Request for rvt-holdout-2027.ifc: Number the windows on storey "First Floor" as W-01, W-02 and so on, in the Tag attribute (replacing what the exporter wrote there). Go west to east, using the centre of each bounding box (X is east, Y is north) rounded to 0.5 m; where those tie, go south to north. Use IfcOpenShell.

First a look at what the model holds.

```python
import ifcopenshell
import ifcopenshell.util.element
import ifcopenshell.util.placement

model = ifcopenshell.open("rvt-holdout-2027.ifc")
print(model.schema)
storey = next(s for s in model.by_type("IfcBuildingStorey") if s.Name == "First Floor")
windows = [e for e in ifcopenshell.util.element.get_decomposition(storey) if e.is_a("IfcWindow")]
for e in sorted(windows, key=lambda e: e.id()):
    origin = ifcopenshell.util.placement.get_local_placement(e.ObjectPlacement)[:3, 3]
    print(e.id(), e.Tag, e.Name, origin.round(2) + 0.0, sep=" | ")
```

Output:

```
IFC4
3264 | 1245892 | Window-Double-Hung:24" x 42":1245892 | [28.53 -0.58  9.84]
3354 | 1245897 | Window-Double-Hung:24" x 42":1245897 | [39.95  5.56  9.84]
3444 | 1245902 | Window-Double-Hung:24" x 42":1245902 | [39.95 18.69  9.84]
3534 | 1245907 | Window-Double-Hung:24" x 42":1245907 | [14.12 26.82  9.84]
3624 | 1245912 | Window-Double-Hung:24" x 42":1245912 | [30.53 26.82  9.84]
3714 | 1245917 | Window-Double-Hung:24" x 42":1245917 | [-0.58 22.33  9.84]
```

```python
import ifcopenshell
import ifcopenshell.geom
import ifcopenshell.util.element
import ifcopenshell.util.shape

model = ifcopenshell.open("rvt-holdout-2027.ifc")
settings = ifcopenshell.geom.settings()
settings.set("use-world-coords", True)


def centre(element):
    shape = ifcopenshell.geom.create_shape(settings, element)
    return ifcopenshell.util.shape.get_bbox_centroid(shape.geometry)


storey = next(s for s in model.by_type("IfcBuildingStorey") if s.Name == "First Floor")
windows = [e for e in ifcopenshell.util.element.get_decomposition(storey) if e.is_a("IfcWindow")]

# Insertion points can sit at a corner or the storey origin, so sort by the geometry (in metres).
centres = {e: centre(e) for e in windows}
windows.sort(key=lambda e: (round(centres[e][0] / 0.5), centres[e][1]))

for i, e in enumerate(windows, start=1):
    number = f"W-{i:02d}"
    e.Tag = number
    print(e.id(), number)

model.write("rvt-holdout-2027_edited.ifc")
```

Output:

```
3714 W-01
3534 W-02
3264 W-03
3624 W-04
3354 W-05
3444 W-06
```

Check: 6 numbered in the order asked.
